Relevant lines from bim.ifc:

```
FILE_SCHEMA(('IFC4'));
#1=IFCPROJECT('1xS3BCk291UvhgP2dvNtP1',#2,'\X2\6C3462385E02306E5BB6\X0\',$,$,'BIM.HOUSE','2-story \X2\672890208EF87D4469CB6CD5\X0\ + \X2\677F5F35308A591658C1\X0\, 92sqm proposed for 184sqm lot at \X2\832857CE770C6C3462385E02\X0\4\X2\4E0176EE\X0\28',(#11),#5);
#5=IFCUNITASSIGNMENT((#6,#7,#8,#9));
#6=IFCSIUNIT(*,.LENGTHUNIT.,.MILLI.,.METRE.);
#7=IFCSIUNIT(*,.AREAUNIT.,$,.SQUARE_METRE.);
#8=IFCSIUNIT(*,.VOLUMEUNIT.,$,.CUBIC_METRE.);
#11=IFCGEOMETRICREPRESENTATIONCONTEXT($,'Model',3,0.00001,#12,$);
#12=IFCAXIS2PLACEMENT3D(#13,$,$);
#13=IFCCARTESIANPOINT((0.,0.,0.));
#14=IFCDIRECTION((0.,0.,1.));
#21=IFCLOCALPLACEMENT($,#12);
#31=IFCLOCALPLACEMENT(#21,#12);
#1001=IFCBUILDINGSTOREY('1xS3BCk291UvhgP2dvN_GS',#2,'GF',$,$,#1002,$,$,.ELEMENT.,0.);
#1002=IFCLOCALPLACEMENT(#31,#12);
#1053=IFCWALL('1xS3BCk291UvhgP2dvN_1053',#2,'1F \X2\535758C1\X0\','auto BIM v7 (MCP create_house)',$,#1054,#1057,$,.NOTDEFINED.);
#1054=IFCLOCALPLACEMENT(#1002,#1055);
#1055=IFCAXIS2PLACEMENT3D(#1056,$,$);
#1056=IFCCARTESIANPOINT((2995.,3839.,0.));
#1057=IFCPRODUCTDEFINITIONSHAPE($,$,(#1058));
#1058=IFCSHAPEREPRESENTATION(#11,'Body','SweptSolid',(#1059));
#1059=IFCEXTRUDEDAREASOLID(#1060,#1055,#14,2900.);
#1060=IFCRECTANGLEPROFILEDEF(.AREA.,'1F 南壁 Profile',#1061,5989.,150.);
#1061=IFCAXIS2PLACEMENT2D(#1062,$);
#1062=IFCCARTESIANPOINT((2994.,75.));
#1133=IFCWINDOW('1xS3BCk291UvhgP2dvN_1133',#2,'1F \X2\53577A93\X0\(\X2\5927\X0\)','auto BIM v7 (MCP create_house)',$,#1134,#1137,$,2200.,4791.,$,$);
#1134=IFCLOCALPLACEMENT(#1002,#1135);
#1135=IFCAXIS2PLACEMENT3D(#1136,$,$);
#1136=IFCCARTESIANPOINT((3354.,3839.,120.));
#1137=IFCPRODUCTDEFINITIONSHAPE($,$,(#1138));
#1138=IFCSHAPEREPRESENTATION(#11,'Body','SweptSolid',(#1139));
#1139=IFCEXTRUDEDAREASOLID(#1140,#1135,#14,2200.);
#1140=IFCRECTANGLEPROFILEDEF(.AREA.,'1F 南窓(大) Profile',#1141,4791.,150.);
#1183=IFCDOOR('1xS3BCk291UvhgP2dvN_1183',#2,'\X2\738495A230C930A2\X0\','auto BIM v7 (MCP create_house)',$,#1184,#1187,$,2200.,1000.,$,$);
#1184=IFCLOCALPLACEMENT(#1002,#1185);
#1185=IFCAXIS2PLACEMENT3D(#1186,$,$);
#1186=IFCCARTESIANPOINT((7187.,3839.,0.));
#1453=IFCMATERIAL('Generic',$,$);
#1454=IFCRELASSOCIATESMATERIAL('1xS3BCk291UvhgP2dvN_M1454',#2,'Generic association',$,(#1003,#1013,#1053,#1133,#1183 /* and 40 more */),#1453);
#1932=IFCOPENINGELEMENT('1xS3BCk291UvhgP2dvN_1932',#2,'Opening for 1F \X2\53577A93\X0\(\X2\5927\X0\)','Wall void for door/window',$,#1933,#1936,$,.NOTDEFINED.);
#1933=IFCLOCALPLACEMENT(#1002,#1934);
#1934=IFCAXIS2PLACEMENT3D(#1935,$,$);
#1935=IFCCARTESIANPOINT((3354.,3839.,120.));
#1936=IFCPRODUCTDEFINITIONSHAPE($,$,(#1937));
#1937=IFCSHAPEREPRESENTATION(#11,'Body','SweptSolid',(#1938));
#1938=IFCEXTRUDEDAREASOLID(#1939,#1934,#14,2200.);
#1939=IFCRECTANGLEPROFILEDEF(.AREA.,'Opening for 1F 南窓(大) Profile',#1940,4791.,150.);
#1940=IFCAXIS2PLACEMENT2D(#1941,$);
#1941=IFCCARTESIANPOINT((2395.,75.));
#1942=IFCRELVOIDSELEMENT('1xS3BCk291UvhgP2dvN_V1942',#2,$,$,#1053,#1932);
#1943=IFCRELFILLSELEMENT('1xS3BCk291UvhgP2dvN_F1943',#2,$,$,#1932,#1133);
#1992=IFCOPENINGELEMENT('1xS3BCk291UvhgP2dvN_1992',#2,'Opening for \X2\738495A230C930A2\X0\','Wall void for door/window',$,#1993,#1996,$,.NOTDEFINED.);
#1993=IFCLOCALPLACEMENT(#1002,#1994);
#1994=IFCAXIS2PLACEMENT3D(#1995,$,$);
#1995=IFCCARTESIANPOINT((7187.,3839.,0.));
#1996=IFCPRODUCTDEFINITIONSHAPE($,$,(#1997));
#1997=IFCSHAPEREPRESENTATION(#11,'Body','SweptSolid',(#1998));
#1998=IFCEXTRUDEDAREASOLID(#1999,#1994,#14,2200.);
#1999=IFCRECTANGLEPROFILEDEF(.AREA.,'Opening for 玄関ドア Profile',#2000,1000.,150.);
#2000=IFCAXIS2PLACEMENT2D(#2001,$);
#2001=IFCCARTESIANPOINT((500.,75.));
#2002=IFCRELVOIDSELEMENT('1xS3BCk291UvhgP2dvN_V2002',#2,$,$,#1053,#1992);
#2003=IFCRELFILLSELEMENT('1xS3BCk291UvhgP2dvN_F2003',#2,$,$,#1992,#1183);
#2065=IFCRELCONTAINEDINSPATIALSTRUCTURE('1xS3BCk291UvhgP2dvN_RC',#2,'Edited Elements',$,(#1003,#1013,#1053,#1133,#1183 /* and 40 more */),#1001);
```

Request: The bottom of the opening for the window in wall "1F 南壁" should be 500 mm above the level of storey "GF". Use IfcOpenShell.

```python
import numpy as np
import ifcopenshell
import ifcopenshell.api.geometry
import ifcopenshell.geom
import ifcopenshell.util.element
import ifcopenshell.util.placement
import ifcopenshell.util.shape
import ifcopenshell.util.unit

model = ifcopenshell.open("bim.ifc")
unit_scale = ifcopenshell.util.unit.calculate_unit_scale(model)

window = model.by_guid("1xS3BCk291UvhgP2dvN_1133")
opening = window.FillsVoids[0].RelatingOpeningElement
storey = ifcopenshell.util.element.get_container(window, ifc_class="IfcBuildingStorey")
level = ifcopenshell.util.placement.get_local_placement(storey.ObjectPlacement)[2, 3]

# The opening's origin need not be at the sill, so measure its lowest point.
shape = ifcopenshell.geom.create_shape(ifcopenshell.geom.settings(), opening)
bottom = ifcopenshell.util.shape.get_shape_bottom_elevation(shape, shape.geometry) / unit_scale
dz = level + 500.0 - bottom

shift = np.array([0.0, 0.0, dz])
# The window is not placed relative to its opening, so move both.
for product in (opening, window):
    matrix = ifcopenshell.util.placement.get_local_placement(product.ObjectPlacement)
    matrix[:3, 3] += shift
    ifcopenshell.api.geometry.edit_object_placement(model, product=product, matrix=matrix, is_si=False)

print(f"moved by {dz * unit_scale:+.3f} m")

model.write("bim_edited.ifc")
```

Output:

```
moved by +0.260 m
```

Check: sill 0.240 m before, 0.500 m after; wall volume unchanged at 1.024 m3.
